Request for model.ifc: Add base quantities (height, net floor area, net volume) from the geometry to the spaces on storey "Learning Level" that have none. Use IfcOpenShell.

First a look at what the model holds.

```python
import ifcopenshell
import ifcopenshell.util.element
import ifcopenshell.util.unit

model = ifcopenshell.open("model.ifc")
print(model.schema)
for unit_type in ("LENGTHUNIT", "AREAUNIT", "VOLUMEUNIT"):
    print(unit_type, ifcopenshell.util.unit.calculate_unit_scale(model, unit_type))
storey = next(s for s in model.by_type("IfcBuildingStorey") if s.Name == "Learning Level")
spaces = [e for e in ifcopenshell.util.element.get_decomposition(storey) if e.is_a("IfcSpace")]
for e in sorted(spaces, key=lambda e: e.id()):
    print(e.id(), e.is_a(), e.Name, list(ifcopenshell.util.element.get_psets(e, qtos_only=True)), sep=" | ")
```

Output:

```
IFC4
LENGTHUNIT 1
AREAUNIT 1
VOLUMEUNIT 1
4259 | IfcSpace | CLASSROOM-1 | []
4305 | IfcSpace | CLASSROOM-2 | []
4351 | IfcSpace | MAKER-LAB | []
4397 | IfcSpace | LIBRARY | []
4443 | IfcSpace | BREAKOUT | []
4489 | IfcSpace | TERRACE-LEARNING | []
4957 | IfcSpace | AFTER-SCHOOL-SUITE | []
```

```python
import ifcopenshell
import ifcopenshell.api.pset
import ifcopenshell.geom
import ifcopenshell.util.element
import ifcopenshell.util.shape
import ifcopenshell.util.unit

model = ifcopenshell.open("model.ifc")
unit_scale = ifcopenshell.util.unit.calculate_unit_scale(model)
area_scale = ifcopenshell.util.unit.calculate_unit_scale(model, "AREAUNIT")
volume_scale = ifcopenshell.util.unit.calculate_unit_scale(model, "VOLUMEUNIT")
settings = ifcopenshell.geom.settings()

storey = next(s for s in model.by_type("IfcBuildingStorey") if s.Name == "Learning Level")
spaces = [e for e in ifcopenshell.util.element.get_decomposition(storey) if e.is_a("IfcSpace")]

for e in sorted(spaces, key=lambda e: e.id()):
    if ifcopenshell.util.element.get_psets(e, qtos_only=True, should_inherit=False):
        continue
    # Geometry comes back in metres, in the element's own axes.
    shape = ifcopenshell.geom.create_shape(settings, e)
    values = {
        "Height": ifcopenshell.util.shape.get_z(shape.geometry) / unit_scale,
        "NetFloorArea": ifcopenshell.util.shape.get_footprint_area(shape.geometry) / area_scale,
        "NetVolume": ifcopenshell.util.shape.get_volume(shape.geometry) / volume_scale,
    }
    qto = ifcopenshell.api.pset.add_qto(model, product=e, name="Qto_SpaceBaseQuantities")
    ifcopenshell.api.pset.edit_qto(model, qto=qto, properties=values)
    print(e.id(), {k: round(v, 3) for k, v in values.items()})

model.write("model_updated.ifc")
```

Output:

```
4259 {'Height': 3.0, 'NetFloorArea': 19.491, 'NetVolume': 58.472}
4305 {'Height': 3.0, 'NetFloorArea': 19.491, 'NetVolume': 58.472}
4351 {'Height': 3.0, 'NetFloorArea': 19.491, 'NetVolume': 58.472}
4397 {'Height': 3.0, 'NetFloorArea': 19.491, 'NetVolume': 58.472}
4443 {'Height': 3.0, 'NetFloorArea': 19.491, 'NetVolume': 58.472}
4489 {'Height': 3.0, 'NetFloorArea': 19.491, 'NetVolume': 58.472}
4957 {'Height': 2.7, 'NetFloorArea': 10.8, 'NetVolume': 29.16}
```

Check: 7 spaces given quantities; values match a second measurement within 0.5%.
